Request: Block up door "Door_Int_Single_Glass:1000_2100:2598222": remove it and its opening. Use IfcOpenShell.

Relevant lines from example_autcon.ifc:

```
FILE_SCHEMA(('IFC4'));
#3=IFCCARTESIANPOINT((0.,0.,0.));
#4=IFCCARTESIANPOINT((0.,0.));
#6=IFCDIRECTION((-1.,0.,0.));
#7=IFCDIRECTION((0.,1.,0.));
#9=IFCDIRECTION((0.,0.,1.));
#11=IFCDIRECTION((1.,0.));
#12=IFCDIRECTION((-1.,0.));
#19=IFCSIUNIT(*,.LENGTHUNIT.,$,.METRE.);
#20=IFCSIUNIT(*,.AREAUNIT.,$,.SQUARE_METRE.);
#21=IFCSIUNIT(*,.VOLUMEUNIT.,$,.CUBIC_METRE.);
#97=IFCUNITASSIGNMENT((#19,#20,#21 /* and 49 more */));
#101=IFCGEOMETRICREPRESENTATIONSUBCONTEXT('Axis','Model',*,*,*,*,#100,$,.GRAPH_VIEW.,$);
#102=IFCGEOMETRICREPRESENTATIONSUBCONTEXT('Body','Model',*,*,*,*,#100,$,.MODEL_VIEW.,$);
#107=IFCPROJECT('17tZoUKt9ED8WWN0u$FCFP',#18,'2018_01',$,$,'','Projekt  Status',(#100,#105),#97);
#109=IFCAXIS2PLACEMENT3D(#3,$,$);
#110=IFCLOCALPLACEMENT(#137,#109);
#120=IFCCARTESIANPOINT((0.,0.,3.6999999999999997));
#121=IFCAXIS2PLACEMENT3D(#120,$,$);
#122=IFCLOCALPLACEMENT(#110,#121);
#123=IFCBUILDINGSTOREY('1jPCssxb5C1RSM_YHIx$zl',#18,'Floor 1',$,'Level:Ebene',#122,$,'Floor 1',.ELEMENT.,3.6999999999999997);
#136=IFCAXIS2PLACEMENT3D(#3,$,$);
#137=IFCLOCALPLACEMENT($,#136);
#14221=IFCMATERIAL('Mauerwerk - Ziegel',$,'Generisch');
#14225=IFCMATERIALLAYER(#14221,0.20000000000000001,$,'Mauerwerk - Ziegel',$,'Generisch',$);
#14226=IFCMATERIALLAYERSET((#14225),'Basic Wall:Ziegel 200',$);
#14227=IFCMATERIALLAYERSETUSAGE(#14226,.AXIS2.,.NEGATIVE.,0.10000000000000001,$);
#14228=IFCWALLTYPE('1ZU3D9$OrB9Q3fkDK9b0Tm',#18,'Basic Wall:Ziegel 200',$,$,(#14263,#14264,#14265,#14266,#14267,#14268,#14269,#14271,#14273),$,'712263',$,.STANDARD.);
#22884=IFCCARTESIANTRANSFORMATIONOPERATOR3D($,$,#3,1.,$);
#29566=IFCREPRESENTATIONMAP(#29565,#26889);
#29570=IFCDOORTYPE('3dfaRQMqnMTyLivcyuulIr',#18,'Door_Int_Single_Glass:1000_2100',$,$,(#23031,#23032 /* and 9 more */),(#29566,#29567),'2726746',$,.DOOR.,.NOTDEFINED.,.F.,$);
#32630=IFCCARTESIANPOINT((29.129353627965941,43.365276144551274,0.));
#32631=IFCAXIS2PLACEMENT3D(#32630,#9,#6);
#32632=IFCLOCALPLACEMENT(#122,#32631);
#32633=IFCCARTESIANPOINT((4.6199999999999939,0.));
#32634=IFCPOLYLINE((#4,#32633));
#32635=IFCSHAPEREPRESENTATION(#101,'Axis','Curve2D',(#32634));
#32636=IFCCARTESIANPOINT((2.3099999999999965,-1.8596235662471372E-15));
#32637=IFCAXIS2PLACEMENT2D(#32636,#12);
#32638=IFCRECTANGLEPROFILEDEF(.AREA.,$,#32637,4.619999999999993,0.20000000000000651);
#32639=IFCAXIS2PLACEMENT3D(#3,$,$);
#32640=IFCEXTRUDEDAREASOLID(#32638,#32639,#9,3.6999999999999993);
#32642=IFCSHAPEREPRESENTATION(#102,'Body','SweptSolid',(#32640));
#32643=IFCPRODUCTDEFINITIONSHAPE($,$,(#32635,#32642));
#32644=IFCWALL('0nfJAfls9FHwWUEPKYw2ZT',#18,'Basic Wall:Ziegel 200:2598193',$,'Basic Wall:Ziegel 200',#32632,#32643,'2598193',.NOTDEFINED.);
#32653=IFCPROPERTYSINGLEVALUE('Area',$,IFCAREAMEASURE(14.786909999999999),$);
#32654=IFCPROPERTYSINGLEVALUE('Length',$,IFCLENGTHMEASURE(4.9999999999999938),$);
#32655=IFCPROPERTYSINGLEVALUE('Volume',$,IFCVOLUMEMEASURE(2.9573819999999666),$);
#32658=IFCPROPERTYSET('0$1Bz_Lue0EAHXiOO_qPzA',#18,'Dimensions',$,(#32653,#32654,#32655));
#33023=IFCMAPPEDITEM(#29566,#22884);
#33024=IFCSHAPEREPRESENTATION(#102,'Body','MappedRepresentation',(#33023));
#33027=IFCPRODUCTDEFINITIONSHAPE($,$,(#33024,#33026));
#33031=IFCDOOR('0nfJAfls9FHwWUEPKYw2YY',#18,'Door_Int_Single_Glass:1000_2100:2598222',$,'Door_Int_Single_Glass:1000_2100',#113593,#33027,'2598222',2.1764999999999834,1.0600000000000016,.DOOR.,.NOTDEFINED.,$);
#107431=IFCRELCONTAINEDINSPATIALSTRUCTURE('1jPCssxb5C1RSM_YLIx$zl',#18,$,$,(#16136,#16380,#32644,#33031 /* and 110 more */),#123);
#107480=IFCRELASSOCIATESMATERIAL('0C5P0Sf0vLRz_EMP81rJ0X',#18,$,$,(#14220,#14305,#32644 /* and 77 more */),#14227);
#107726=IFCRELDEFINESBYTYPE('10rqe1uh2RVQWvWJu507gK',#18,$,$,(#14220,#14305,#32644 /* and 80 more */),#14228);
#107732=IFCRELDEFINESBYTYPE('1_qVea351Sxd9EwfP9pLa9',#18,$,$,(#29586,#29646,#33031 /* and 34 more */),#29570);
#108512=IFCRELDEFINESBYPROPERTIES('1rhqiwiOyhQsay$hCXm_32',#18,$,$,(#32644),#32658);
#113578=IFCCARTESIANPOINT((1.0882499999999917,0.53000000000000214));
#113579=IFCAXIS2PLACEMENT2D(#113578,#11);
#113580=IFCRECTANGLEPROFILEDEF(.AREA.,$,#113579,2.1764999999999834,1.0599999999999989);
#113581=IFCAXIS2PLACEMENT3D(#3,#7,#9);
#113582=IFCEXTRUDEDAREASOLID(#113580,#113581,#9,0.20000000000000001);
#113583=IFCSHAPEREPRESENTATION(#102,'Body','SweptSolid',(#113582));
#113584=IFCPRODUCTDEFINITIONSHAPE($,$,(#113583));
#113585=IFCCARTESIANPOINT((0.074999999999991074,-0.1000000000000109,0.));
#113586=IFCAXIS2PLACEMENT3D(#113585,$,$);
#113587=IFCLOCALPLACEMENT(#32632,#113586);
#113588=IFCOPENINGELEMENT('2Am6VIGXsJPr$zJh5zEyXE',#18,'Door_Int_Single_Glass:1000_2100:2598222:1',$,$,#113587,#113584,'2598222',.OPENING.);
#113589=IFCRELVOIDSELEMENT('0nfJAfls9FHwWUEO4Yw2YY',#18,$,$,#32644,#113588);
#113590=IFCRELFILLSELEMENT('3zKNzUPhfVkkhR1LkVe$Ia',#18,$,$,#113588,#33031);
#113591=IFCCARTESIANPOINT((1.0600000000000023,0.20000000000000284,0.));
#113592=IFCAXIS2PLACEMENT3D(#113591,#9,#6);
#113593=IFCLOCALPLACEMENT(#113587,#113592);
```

```python
import ifcopenshell
import ifcopenshell.api.feature
import ifcopenshell.api.pset
import ifcopenshell.api.root
import ifcopenshell.geom
import ifcopenshell.util.element
import ifcopenshell.util.shape
import ifcopenshell.util.unit

model = ifcopenshell.open("example_autcon.ifc")
area_scale = ifcopenshell.util.unit.calculate_unit_scale(model, "AREAUNIT")
volume_scale = ifcopenshell.util.unit.calculate_unit_scale(model, "VOLUMEUNIT")
settings = ifcopenshell.geom.settings()


def volume(element):
    """Net volume in cubic metres, openings subtracted."""
    shape = ifcopenshell.geom.create_shape(settings, element)
    return ifcopenshell.util.shape.get_volume(shape.geometry)


door = model.by_id(33031)
opening = door.FillsVoids[0].RelatingOpeningElement
wall = opening.VoidsElements[0].RelatingBuildingElement
before = volume(wall)

ifcopenshell.api.root.remove_product(model, product=door)
ifcopenshell.api.feature.remove_feature(model, feature=opening)

after = volume(wall)
thickness = 0.2  # wall thickness in metres

# Update the wall's stored quantities.
pset = model.by_id(ifcopenshell.util.element.get_pset(wall, "Dimensions", should_inherit=False)["id"])
ifcopenshell.api.pset.edit_pset(model, pset=pset, properties={
    "Area": model.create_entity("IfcAreaMeasure", after / thickness / area_scale),
    "Volume": model.create_entity("IfcVolumeMeasure", after / volume_scale),
})

print(f"wall volume {before:.3f} -> {after:.3f} m3")

model.write("example_autcon_edited.ifc")
```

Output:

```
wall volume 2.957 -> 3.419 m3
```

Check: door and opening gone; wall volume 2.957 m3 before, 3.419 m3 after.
